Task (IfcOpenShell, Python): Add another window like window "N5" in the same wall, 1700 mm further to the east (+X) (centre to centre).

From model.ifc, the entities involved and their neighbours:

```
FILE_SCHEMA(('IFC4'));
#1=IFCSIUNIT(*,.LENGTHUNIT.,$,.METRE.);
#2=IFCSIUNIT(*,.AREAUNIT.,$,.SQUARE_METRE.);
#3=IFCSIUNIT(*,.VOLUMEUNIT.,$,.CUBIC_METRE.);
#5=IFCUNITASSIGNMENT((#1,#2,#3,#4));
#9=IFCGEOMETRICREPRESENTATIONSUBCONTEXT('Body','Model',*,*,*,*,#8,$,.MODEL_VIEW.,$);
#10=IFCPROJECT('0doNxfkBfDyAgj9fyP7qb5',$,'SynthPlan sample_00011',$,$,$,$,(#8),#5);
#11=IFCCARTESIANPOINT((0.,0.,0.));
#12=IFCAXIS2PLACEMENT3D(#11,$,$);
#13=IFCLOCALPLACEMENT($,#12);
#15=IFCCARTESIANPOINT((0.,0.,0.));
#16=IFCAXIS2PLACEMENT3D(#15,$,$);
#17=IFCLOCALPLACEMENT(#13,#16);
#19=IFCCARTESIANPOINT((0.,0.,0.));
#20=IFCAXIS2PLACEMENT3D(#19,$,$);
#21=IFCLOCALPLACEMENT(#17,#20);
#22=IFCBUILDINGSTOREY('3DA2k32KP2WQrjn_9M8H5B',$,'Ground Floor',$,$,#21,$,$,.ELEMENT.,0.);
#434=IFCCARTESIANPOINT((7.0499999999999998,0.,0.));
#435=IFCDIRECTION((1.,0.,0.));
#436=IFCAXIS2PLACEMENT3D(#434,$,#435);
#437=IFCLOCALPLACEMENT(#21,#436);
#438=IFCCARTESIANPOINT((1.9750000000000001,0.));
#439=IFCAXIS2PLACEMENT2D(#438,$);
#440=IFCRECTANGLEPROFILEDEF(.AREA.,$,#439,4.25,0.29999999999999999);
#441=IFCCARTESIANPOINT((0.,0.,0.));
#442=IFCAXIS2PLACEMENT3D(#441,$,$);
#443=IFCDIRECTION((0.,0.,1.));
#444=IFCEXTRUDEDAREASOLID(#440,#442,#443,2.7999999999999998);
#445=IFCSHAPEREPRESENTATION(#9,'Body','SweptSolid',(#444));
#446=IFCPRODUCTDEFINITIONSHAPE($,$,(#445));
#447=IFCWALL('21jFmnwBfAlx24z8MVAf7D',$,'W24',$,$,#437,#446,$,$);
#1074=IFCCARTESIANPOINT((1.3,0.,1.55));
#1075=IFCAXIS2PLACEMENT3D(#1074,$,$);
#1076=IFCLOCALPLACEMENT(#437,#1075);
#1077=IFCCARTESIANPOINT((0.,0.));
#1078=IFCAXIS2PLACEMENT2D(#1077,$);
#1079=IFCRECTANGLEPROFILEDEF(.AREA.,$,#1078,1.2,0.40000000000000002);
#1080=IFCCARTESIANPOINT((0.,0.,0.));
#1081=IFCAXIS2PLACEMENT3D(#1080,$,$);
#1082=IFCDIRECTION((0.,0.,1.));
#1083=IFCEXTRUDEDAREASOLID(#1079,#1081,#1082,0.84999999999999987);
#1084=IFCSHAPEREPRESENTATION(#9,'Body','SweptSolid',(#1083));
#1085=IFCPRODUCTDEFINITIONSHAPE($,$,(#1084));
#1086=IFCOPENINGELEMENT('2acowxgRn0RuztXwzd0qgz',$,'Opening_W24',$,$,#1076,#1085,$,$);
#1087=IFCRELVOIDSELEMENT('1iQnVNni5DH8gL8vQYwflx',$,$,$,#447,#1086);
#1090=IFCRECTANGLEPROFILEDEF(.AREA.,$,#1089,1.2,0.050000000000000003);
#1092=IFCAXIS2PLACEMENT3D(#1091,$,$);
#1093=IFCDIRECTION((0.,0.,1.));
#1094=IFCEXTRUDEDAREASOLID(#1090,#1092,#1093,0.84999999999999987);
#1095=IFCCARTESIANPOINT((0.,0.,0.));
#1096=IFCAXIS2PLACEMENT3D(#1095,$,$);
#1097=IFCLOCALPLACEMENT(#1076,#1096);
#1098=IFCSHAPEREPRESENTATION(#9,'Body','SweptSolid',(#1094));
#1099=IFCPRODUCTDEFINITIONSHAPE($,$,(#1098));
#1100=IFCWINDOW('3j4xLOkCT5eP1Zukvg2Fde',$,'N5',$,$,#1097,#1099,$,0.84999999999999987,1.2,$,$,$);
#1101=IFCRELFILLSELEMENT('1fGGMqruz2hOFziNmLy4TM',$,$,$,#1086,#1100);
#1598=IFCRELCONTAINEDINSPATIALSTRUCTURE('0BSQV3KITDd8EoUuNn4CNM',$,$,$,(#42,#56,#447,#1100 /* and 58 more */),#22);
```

```python
import ifcopenshell
import ifcopenshell.api.feature
import ifcopenshell.api.geometry
import ifcopenshell.api.root
import ifcopenshell.geom
import ifcopenshell.util.element
import ifcopenshell.util.placement
import ifcopenshell.util.shape
import ifcopenshell.util.unit

model = ifcopenshell.open("model.ifc")
unit_scale = ifcopenshell.util.unit.calculate_unit_scale(model)
settings = ifcopenshell.geom.settings()


def volume(element):
    """Net volume in cubic metres, openings subtracted."""
    shape = ifcopenshell.geom.create_shape(settings, element)
    return ifcopenshell.util.shape.get_volume(shape.geometry)


window = model.by_id(1100)
opening = window.FillsVoids[0].RelatingOpeningElement
wall = opening.VoidsElements[0].RelatingBuildingElement
before = volume(wall)
shift = ifcopenshell.util.placement.get_local_placement(wall.ObjectPlacement)[:3, 0] * 1.7 / unit_scale

# copy_class copies the void relationship, type, container and properties, but no geometry.
new_opening = ifcopenshell.api.root.copy_class(model, product=opening)
new_opening.Representation = ifcopenshell.util.element.copy_deep(
    model, opening.Representation, exclude=["IfcGeometricRepresentationContext", "IfcRepresentationMap"]
)
new_window = ifcopenshell.api.root.copy_class(model, product=window)
new_window.Representation = ifcopenshell.util.element.copy_deep(
    model, window.Representation, exclude=["IfcGeometricRepresentationContext", "IfcRepresentationMap"]
)
ifcopenshell.api.feature.add_filling(model, opening=new_opening, element=new_window)

for old, new in ((opening, new_opening), (window, new_window)):
    matrix = ifcopenshell.util.placement.get_local_placement(old.ObjectPlacement)
    matrix[:3, 3] += shift
    ifcopenshell.api.geometry.edit_object_placement(model, product=new, matrix=matrix, is_si=False)

after = volume(wall)

print(f"wall volume {before:.3f} -> {after:.3f} m3")

model.write("model_v2.ifc")
```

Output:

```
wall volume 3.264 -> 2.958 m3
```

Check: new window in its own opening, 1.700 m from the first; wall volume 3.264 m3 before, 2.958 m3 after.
